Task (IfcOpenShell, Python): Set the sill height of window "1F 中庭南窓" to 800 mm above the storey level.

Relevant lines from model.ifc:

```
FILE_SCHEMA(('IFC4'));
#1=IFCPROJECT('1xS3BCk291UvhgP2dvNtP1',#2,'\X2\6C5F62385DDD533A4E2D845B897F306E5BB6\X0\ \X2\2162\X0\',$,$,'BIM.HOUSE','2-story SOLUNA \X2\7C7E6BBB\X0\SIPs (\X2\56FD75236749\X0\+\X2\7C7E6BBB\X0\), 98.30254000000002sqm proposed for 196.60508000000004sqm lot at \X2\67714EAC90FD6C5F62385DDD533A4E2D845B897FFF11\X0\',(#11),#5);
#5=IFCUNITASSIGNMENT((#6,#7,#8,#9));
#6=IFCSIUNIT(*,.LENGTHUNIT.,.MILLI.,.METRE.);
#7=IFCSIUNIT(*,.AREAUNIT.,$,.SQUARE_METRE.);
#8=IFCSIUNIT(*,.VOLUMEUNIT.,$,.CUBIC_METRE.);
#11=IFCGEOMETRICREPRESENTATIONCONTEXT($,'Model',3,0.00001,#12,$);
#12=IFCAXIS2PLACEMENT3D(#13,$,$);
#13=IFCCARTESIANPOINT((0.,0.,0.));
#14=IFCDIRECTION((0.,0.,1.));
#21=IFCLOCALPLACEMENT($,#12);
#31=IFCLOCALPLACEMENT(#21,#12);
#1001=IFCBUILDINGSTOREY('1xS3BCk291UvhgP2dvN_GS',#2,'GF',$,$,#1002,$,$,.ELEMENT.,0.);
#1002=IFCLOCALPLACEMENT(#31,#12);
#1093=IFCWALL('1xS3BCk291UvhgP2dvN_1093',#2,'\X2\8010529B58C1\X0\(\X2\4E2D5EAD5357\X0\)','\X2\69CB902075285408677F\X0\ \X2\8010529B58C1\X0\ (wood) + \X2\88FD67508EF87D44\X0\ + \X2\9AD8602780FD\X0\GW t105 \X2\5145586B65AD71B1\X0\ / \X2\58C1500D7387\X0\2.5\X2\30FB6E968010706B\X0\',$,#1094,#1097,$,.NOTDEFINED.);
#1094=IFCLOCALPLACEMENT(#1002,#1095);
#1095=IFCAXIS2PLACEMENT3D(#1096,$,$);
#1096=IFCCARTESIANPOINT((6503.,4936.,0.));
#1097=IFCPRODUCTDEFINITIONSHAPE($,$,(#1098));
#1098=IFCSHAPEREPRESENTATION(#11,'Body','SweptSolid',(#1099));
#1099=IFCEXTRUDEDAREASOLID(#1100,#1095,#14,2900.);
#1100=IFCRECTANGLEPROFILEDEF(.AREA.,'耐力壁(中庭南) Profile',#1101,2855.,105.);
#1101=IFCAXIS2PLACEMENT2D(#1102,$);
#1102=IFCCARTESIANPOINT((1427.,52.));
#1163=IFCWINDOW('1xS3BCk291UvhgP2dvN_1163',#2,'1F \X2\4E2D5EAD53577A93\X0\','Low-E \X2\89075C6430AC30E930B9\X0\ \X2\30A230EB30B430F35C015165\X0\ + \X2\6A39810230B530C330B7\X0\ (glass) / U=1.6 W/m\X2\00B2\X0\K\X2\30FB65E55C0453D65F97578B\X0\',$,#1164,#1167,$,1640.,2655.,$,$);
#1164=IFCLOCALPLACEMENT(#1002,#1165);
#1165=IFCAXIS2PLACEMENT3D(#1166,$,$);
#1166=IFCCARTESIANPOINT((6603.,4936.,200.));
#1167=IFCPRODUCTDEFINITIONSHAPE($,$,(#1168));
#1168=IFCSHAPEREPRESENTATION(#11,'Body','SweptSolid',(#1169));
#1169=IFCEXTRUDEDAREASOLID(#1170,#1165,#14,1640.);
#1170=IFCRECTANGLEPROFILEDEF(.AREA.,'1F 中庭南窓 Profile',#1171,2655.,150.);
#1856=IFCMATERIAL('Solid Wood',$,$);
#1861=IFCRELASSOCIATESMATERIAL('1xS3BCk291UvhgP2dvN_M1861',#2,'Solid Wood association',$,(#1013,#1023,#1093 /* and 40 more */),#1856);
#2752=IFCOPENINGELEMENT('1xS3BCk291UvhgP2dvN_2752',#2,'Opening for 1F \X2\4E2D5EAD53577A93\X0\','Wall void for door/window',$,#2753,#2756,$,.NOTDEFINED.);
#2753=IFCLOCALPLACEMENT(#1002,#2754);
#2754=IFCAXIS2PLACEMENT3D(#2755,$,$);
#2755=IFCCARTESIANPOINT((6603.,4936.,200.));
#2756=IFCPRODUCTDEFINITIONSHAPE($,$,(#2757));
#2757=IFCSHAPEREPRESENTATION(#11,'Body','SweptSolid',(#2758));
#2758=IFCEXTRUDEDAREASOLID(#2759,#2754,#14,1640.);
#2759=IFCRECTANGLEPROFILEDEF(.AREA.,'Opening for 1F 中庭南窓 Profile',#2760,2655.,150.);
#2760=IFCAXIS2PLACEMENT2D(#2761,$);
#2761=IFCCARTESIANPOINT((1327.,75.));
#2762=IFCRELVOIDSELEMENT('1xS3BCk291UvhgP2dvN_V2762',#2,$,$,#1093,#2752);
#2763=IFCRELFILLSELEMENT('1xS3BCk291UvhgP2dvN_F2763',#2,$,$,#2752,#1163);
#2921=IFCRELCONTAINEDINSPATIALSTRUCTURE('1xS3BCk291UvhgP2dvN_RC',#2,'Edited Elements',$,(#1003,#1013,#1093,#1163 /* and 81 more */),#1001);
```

```python
import numpy as np
import ifcopenshell
import ifcopenshell.api.geometry
import ifcopenshell.geom
import ifcopenshell.util.element
import ifcopenshell.util.placement
import ifcopenshell.util.shape
import ifcopenshell.util.unit

model = ifcopenshell.open("model.ifc")
unit_scale = ifcopenshell.util.unit.calculate_unit_scale(model)

window = model.by_id(1163)
opening = window.FillsVoids[0].RelatingOpeningElement
storey = ifcopenshell.util.element.get_container(window, ifc_class="IfcBuildingStorey")
level = ifcopenshell.util.placement.get_local_placement(storey.ObjectPlacement)[2, 3]

# The opening's origin need not be at the sill, so measure its lowest point.
shape = ifcopenshell.geom.create_shape(ifcopenshell.geom.settings(), opening)
bottom = ifcopenshell.util.shape.get_shape_bottom_elevation(shape, shape.geometry) / unit_scale
dz = level + 0.8 / unit_scale - bottom

shift = np.array([0.0, 0.0, dz])
# The window is not placed relative to its opening, so move both.
for product in (opening, window):
    matrix = ifcopenshell.util.placement.get_local_placement(product.ObjectPlacement)
    matrix[:3, 3] += shift
    ifcopenshell.api.geometry.edit_object_placement(model, product=product, matrix=matrix, is_si=False)

print(f"moved by {dz * unit_scale:+.3f} m")

model.write("model_rev.ifc")
```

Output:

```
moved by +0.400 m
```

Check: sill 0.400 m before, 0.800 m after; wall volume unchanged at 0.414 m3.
